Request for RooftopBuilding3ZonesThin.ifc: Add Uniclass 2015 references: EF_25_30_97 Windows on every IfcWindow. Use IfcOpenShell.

First a look at what the model holds.

```python
import ifcopenshell

model = ifcopenshell.open("RooftopBuilding3ZonesThin.ifc")
print(model.schema)
print("classifications:", [c.Name for c in model.by_type("IfcClassification")])
for ifc_class in ("IfcDoor", "IfcRoof", "IfcStair", "IfcWall", "IfcWindow"):
    print(ifc_class, len(model.by_type(ifc_class)))
```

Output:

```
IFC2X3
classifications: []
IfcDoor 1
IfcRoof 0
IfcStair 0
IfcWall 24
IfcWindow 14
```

```python
import ifcopenshell
import ifcopenshell.api.classification

model = ifcopenshell.open("RooftopBuilding3ZonesThin.ifc")

# IFC2X3 requires Source and Edition and has no link from the project to the system.
system = model.create_entity("IfcClassification", Source="NBS", Edition="2015", Name="Uniclass 2015")

codes = {
    "IfcWindow": ("EF_25_30_97", "Windows"),
}
for ifc_class, (code, name) in codes.items():
    products = model.by_type(ifc_class)
    ifcopenshell.api.classification.add_reference(
        model, products=products, classification=system, identification=code, name=name
    )
    print(code, len(products))

model.write("RooftopBuilding3ZonesThin_rev.ifc")
```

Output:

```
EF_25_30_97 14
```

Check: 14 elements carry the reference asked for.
